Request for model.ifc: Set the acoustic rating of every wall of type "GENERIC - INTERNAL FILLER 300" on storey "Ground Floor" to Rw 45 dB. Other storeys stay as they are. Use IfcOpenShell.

First a look at what the model holds.

```python
import ifcopenshell
import ifcopenshell.util.element

model = ifcopenshell.open("model.ifc")
print(model.schema)
storey = next(s for s in model.by_type("IfcBuildingStorey") if s.Name == "Ground Floor")
walls = [e for e in ifcopenshell.util.element.get_decomposition(storey) if e.is_a("IfcWall")]
seen = {}
for e in walls:
    element_type = ifcopenshell.util.element.get_type(e)
    key = (element_type.Name if element_type != e and element_type else None, ifcopenshell.util.element.get_pset(e, "Pset_WallCommon", "AcousticRating"))
    seen[key] = seen.get(key, 0) + 1
for (name, value), count in sorted(seen.items(), key=str):
    print(count, "x", name, "|", value)
```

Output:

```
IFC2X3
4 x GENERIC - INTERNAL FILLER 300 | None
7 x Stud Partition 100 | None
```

```python
import ifcopenshell
import ifcopenshell.api.pset
import ifcopenshell.util.element

model = ifcopenshell.open("model.ifc")

storey = next(s for s in model.by_type("IfcBuildingStorey") if s.Name == "Ground Floor")
walls = [e for e in ifcopenshell.util.element.get_decomposition(storey) if e.is_a("IfcWall")]

count = 0
for e in walls:
    element_type = ifcopenshell.util.element.get_type(e)
    if element_type in (None, e) or element_type.Name != "GENERIC - INTERNAL FILLER 300":
        continue
    # add_pset returns the element's existing set when there is one.
    pset = ifcopenshell.api.pset.add_pset(model, product=e, name="Pset_WallCommon")
    ifcopenshell.api.pset.edit_pset(model, pset=pset, properties={"AcousticRating": "Rw 45 dB"})
    count += 1

print(count, "walls updated")

model.write("model-out.ifc")
```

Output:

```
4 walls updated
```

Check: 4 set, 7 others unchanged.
